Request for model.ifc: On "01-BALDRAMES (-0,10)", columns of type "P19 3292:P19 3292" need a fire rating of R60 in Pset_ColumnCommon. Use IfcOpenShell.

First a look at what the model holds.

```python
import ifcopenshell
import ifcopenshell.util.element

model = ifcopenshell.open("model.ifc")
print(model.schema)
storey = next(s for s in model.by_type("IfcBuildingStorey") if s.Name == "01-BALDRAMES (-0,10)")
columns = [e for e in ifcopenshell.util.element.get_decomposition(storey) if e.is_a("IfcColumn")]
seen = {}
for e in columns:
    element_type = ifcopenshell.util.element.get_type(e)
    key = (element_type.Name if element_type != e and element_type else None, ifcopenshell.util.element.get_pset(e, "Pset_ColumnCommon", "FireRating"))
    seen[key] = seen.get(key, 0) + 1
for (name, value), count in sorted(seen.items(), key=str):
    print(count, "x", name, "|", value)
```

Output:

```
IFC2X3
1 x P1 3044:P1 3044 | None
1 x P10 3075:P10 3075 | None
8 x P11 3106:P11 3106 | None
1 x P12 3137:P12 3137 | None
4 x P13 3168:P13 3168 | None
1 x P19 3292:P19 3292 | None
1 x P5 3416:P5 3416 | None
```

```python
import ifcopenshell
import ifcopenshell.api.pset
import ifcopenshell.util.element

model = ifcopenshell.open("model.ifc")

storey = next(s for s in model.by_type("IfcBuildingStorey") if s.Name == "01-BALDRAMES (-0,10)")
columns = [e for e in ifcopenshell.util.element.get_decomposition(storey) if e.is_a("IfcColumn")]

count = 0
for e in columns:
    element_type = ifcopenshell.util.element.get_type(e)
    if element_type in (None, e) or element_type.Name != "P19 3292:P19 3292":
        continue
    # add_pset returns the element's existing set when there is one.
    pset = ifcopenshell.api.pset.add_pset(model, product=e, name="Pset_ColumnCommon")
    ifcopenshell.api.pset.edit_pset(model, pset=pset, properties={"FireRating": "R60"})
    count += 1

print(count, "columns updated")

model.write("model_updated.ifc")
```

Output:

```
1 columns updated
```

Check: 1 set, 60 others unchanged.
